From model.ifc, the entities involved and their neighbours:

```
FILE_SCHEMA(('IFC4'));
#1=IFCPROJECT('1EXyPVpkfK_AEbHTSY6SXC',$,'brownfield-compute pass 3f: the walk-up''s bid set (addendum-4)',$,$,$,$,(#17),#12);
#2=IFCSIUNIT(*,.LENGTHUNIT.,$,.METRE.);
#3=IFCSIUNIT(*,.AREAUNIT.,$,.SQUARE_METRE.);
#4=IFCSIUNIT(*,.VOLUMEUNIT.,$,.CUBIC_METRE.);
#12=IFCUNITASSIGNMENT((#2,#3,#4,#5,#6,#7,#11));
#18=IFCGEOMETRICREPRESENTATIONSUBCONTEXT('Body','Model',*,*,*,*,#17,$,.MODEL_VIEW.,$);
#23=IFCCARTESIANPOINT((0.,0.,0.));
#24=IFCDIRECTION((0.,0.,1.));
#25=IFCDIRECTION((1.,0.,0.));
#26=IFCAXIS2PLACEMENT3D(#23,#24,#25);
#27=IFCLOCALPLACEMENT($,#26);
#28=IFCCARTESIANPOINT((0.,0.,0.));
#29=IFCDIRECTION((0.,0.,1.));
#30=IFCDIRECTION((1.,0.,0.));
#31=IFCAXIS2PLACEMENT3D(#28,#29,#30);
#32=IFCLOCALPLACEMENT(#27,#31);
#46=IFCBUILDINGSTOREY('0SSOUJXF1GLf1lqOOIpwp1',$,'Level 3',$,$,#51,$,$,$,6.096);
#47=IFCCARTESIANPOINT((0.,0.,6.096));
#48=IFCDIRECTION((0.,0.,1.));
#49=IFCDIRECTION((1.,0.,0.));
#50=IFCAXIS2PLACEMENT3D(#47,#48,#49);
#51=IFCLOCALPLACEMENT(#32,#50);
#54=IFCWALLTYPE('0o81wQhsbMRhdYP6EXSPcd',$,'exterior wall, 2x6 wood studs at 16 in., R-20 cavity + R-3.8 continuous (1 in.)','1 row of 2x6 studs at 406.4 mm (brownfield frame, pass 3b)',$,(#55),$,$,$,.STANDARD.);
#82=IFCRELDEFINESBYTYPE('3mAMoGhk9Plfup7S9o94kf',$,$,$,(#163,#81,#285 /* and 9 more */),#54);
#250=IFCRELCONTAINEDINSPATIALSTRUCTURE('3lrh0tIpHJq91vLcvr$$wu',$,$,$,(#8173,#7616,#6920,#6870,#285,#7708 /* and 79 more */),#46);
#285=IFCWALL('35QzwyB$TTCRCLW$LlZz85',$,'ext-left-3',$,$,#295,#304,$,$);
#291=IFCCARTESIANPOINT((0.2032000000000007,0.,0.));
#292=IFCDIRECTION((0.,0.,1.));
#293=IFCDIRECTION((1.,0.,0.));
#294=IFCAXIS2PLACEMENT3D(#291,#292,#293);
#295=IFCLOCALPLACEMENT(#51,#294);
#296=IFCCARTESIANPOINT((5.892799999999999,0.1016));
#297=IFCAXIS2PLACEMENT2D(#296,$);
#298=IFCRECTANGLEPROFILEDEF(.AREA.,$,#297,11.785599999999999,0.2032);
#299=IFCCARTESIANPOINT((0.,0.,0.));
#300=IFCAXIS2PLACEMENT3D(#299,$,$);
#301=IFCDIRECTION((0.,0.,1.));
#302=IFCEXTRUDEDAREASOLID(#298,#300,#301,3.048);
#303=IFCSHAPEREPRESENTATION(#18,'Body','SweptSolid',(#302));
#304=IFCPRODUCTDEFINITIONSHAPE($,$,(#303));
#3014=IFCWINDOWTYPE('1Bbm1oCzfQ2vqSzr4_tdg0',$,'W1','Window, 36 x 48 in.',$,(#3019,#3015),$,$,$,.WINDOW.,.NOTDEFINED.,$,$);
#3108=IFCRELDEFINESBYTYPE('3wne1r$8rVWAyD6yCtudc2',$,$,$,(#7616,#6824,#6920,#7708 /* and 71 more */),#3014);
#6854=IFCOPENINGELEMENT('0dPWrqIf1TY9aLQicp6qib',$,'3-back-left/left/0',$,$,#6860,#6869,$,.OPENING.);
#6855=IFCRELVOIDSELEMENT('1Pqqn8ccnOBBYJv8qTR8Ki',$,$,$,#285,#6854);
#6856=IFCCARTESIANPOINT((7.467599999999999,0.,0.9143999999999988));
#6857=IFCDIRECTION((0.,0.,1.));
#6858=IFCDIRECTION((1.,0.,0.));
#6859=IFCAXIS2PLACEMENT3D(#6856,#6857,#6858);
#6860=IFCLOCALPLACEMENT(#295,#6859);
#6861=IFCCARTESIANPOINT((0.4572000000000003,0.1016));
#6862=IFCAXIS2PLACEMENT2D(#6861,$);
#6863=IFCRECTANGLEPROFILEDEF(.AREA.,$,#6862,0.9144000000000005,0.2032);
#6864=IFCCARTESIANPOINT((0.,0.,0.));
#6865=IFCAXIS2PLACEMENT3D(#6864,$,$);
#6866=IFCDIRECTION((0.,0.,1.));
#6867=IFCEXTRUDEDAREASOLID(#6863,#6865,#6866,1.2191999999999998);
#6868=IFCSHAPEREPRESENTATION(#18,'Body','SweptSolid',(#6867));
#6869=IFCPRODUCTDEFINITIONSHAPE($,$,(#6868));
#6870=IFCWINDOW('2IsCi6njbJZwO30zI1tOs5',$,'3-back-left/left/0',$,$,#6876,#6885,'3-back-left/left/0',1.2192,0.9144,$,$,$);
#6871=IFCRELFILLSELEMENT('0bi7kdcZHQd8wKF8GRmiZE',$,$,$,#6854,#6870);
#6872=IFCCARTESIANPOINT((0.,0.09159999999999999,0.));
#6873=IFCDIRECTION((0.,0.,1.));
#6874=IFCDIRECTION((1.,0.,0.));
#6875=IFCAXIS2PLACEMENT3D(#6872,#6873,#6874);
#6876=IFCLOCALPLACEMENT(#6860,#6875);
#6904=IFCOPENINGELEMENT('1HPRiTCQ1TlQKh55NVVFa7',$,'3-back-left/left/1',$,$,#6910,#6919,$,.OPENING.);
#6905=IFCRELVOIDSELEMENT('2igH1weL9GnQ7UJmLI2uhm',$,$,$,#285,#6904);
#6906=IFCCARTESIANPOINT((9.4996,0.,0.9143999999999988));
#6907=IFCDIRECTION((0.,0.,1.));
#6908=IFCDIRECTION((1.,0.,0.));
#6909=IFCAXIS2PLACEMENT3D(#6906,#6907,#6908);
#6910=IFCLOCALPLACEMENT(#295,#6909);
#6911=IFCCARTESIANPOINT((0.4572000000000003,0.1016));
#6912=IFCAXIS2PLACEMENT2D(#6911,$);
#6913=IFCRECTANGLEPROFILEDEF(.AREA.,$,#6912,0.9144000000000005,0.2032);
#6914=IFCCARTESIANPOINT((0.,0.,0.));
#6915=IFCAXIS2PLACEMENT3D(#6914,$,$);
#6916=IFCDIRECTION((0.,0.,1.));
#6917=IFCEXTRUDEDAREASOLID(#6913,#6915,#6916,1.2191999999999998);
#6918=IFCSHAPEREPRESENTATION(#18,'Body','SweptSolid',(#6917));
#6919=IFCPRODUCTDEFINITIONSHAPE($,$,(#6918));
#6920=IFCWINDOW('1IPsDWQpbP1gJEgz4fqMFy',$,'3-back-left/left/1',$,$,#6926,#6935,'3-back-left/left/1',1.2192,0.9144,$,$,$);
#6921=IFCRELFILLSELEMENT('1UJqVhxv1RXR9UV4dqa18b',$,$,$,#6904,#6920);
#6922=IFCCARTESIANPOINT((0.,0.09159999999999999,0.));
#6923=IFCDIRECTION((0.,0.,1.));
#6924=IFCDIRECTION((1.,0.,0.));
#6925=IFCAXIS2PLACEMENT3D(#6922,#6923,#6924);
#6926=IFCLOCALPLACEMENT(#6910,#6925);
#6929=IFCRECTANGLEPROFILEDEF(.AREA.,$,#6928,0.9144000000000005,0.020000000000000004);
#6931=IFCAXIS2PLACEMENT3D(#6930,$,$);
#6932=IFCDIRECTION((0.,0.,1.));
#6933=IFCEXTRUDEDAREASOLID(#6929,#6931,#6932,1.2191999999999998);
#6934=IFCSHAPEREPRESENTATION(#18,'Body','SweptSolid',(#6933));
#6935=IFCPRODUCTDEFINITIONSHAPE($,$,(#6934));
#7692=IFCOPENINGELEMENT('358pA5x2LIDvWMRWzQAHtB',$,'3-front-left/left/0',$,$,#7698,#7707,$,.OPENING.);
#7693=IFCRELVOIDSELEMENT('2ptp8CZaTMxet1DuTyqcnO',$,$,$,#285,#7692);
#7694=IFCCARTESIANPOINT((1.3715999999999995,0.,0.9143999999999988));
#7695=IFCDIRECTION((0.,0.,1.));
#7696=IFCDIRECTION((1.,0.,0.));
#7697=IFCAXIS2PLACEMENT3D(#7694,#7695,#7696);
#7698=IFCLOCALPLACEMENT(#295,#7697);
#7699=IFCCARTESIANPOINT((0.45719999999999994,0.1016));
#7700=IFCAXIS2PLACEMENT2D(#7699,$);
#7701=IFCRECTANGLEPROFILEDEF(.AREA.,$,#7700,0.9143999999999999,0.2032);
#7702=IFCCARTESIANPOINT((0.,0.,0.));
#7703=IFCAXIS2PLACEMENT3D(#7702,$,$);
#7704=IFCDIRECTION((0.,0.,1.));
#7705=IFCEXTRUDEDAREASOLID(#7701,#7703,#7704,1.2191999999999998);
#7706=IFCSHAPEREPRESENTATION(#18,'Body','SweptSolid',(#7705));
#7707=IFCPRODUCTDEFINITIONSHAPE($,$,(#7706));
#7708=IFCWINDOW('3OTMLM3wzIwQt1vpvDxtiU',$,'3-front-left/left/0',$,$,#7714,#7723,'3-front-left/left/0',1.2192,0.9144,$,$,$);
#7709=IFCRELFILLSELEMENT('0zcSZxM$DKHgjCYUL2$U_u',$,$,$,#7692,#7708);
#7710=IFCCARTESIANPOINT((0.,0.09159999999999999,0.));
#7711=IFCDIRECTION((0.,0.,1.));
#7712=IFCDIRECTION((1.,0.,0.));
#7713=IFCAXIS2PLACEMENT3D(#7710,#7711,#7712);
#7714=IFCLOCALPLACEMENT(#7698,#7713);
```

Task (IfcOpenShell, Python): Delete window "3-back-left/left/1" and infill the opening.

```python
import ifcopenshell
import ifcopenshell.api.feature
import ifcopenshell.api.root
import ifcopenshell.geom
import ifcopenshell.util.shape

model = ifcopenshell.open("model.ifc")
settings = ifcopenshell.geom.settings()


def volume(element):
    """Net volume in cubic metres, openings subtracted."""
    shape = ifcopenshell.geom.create_shape(settings, element)
    return ifcopenshell.util.shape.get_volume(shape.geometry)


window = model.by_id(6920)
opening = window.FillsVoids[0].RelatingOpeningElement
wall = opening.VoidsElements[0].RelatingBuildingElement
before = volume(wall)

ifcopenshell.api.root.remove_product(model, product=window)
ifcopenshell.api.feature.remove_feature(model, feature=opening)

after = volume(wall)

print(f"wall volume {before:.3f} -> {after:.3f} m3")

model.write("model_rev.ifc")
```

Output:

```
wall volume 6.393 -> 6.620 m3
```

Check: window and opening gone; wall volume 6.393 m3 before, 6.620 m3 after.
